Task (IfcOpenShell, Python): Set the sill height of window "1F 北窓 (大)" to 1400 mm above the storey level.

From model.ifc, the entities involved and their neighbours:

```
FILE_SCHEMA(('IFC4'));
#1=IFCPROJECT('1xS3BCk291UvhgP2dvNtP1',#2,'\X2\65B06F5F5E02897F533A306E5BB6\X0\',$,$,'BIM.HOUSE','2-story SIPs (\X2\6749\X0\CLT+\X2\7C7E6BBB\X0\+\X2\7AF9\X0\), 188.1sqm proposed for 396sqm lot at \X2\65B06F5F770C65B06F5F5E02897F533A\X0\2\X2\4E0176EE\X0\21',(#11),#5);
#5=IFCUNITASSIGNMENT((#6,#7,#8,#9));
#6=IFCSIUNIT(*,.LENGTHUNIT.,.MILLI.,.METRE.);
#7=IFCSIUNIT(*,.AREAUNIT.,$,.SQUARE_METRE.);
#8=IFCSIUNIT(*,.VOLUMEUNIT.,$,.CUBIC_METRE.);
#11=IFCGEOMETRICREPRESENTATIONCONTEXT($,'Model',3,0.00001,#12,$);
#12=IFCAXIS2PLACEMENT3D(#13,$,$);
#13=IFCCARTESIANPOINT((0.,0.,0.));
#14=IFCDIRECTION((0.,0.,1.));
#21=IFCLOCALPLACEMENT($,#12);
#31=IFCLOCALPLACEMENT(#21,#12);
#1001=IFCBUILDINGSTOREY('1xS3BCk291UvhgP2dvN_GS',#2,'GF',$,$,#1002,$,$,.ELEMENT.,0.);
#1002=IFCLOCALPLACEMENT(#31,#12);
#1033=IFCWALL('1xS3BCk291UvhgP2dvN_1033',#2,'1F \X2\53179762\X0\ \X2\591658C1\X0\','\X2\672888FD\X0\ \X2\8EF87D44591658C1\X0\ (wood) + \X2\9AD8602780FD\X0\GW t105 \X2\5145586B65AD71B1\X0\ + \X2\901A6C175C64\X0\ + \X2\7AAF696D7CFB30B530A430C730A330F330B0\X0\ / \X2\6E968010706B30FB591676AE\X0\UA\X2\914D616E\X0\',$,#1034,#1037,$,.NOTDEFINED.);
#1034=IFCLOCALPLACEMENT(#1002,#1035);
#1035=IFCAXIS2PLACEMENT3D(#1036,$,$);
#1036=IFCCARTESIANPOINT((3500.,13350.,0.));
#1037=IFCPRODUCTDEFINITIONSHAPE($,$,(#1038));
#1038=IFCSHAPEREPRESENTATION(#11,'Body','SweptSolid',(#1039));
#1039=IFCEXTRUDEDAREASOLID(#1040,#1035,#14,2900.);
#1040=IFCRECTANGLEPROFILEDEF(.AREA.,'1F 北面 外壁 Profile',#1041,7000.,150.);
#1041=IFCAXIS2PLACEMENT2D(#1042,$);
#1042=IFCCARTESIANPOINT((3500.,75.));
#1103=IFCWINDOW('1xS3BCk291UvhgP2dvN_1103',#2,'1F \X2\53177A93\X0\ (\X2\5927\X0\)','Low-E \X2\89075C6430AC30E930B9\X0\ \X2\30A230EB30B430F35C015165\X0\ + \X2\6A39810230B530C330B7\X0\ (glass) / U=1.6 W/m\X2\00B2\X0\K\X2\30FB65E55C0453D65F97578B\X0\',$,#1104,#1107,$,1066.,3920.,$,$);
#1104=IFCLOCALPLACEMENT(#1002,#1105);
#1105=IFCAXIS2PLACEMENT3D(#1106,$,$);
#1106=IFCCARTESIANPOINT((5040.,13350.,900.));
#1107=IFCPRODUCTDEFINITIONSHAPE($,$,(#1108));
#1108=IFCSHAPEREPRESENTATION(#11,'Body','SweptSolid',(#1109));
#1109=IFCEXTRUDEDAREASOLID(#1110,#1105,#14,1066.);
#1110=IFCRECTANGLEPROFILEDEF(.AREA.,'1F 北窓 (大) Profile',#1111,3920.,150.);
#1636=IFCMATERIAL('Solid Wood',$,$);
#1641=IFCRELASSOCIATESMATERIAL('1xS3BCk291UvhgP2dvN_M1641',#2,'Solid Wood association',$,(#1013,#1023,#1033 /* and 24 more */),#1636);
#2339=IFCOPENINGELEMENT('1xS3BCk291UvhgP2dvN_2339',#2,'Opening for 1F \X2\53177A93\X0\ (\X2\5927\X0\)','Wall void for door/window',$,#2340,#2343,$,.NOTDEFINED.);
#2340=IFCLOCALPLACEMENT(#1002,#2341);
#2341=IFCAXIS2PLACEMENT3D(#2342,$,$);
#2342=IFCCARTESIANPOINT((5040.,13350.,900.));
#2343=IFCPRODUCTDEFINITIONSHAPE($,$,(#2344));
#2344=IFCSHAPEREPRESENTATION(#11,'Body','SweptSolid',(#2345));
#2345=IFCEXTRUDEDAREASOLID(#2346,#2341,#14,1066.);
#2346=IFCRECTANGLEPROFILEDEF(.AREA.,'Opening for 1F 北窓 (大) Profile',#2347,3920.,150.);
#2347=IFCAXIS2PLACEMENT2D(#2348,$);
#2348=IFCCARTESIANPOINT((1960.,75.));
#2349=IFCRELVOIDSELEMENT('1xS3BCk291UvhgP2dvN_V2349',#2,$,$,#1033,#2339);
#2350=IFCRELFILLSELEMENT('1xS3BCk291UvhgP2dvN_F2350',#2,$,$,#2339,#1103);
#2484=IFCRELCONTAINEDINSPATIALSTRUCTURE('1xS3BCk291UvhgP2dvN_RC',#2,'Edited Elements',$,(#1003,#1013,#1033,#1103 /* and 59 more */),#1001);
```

```python
import numpy as np
import ifcopenshell
import ifcopenshell.api.geometry
import ifcopenshell.geom
import ifcopenshell.util.element
import ifcopenshell.util.placement
import ifcopenshell.util.shape
import ifcopenshell.util.unit

model = ifcopenshell.open("model.ifc")
unit_scale = ifcopenshell.util.unit.calculate_unit_scale(model)

window = model.by_guid("1xS3BCk291UvhgP2dvN_1103")
opening = window.FillsVoids[0].RelatingOpeningElement
storey = ifcopenshell.util.element.get_container(window, ifc_class="IfcBuildingStorey")
level = ifcopenshell.util.placement.get_local_placement(storey.ObjectPlacement)[2, 3]

# The opening's origin need not be at the sill, so measure its lowest point.
shape = ifcopenshell.geom.create_shape(ifcopenshell.geom.settings(), opening)
bottom = ifcopenshell.util.shape.get_shape_bottom_elevation(shape, shape.geometry) / unit_scale
dz = level + 1400.0 - bottom

shift = np.array([0.0, 0.0, dz])
# The window is not placed relative to its opening, so move both.
for product in (opening, window):
    matrix = ifcopenshell.util.placement.get_local_placement(product.ObjectPlacement)
    matrix[:3, 3] += shift
    ifcopenshell.api.geometry.edit_object_placement(model, product=product, matrix=matrix, is_si=False)

print(f"moved by {dz * unit_scale:+.3f} m")

model.write("model_updated.ifc")
```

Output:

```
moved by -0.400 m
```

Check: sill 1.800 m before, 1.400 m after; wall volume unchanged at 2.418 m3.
